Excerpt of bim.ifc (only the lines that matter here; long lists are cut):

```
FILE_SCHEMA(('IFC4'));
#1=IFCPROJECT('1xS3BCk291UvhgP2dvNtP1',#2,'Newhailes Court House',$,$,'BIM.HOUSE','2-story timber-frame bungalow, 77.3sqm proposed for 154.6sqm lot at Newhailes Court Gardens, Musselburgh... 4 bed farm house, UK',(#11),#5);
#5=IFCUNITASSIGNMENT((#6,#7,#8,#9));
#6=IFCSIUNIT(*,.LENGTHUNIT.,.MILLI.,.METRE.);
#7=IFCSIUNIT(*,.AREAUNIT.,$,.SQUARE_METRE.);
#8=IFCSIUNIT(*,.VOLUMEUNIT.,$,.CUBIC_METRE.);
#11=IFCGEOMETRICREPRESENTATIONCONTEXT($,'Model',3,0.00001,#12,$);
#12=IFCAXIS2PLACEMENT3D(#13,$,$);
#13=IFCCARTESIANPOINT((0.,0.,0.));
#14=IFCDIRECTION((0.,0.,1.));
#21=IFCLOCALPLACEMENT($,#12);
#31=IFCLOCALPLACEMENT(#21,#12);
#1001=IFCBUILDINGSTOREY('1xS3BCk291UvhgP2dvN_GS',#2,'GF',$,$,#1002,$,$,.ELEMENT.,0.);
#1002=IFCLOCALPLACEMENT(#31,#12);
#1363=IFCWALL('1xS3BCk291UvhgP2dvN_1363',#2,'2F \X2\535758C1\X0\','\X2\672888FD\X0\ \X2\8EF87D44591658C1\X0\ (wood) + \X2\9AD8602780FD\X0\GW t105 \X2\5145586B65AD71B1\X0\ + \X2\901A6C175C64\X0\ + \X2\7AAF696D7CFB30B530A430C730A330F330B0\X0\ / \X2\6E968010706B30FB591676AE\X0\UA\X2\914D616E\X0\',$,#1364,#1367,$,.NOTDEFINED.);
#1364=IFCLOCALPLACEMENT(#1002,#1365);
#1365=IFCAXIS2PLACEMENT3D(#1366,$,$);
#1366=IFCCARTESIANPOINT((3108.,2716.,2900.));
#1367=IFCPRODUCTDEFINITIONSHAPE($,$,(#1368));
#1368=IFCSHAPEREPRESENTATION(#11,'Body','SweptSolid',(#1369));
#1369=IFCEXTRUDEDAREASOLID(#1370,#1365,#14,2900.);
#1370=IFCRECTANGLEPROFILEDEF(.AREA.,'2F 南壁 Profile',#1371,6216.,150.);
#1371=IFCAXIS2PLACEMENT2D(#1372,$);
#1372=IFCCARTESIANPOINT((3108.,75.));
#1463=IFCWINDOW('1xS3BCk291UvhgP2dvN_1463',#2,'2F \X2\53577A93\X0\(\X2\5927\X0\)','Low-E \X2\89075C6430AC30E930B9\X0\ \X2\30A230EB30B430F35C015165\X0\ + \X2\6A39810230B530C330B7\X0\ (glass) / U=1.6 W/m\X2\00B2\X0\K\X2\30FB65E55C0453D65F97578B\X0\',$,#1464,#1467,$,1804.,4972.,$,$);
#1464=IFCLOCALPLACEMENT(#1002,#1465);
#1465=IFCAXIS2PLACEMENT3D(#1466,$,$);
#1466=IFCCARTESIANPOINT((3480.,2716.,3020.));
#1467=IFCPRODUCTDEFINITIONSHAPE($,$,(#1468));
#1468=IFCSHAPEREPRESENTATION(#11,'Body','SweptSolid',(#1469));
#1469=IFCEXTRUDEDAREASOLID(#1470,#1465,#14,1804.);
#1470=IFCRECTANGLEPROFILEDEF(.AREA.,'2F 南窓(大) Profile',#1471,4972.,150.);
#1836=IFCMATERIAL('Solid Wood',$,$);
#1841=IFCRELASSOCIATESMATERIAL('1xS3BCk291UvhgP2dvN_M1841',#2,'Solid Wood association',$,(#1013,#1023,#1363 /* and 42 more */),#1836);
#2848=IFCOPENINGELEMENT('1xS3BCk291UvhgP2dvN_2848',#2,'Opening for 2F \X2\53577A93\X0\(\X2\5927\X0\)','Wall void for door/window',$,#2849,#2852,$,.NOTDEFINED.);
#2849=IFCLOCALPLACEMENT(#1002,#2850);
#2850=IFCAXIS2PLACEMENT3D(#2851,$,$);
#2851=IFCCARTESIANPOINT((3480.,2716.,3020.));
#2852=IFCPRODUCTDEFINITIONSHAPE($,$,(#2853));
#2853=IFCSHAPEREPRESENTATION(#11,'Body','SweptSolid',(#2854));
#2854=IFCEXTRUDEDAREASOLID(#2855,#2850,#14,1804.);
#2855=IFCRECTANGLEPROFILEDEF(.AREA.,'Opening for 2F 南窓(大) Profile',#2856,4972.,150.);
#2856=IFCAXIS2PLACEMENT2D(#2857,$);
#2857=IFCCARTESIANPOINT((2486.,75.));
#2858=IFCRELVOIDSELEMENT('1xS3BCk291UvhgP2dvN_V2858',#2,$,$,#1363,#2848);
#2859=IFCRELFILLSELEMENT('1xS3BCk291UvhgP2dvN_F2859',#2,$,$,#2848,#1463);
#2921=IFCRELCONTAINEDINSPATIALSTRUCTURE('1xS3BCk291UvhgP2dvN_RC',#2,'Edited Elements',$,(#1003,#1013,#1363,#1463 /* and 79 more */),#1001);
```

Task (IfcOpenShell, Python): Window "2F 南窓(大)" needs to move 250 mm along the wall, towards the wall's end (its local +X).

```python
import ifcopenshell
import ifcopenshell.api.geometry
import ifcopenshell.util.placement
import ifcopenshell.util.unit

model = ifcopenshell.open("bim.ifc")
unit_scale = ifcopenshell.util.unit.calculate_unit_scale(model)

window = model.by_id(1463)
opening = window.FillsVoids[0].RelatingOpeningElement
wall = opening.VoidsElements[0].RelatingBuildingElement

wall_matrix = ifcopenshell.util.placement.get_local_placement(wall.ObjectPlacement)
shift = wall_matrix[:3, 0] * 0.25 / unit_scale
before = ifcopenshell.util.placement.get_local_placement(window.ObjectPlacement)[:3, 3].copy()

# The window is not placed relative to its opening, so move both.
for product in (opening, window):
    matrix = ifcopenshell.util.placement.get_local_placement(product.ObjectPlacement)
    matrix[:3, 3] += shift
    ifcopenshell.api.geometry.edit_object_placement(model, product=product, matrix=matrix, is_si=False)

after = ifcopenshell.util.placement.get_local_placement(window.ObjectPlacement)[:3, 3]
print("window moved by", (after - before).round(3) + 0.0)

model.write("bim_v2.ifc")
```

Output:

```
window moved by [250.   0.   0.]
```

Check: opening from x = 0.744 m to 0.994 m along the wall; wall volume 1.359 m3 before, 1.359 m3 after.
